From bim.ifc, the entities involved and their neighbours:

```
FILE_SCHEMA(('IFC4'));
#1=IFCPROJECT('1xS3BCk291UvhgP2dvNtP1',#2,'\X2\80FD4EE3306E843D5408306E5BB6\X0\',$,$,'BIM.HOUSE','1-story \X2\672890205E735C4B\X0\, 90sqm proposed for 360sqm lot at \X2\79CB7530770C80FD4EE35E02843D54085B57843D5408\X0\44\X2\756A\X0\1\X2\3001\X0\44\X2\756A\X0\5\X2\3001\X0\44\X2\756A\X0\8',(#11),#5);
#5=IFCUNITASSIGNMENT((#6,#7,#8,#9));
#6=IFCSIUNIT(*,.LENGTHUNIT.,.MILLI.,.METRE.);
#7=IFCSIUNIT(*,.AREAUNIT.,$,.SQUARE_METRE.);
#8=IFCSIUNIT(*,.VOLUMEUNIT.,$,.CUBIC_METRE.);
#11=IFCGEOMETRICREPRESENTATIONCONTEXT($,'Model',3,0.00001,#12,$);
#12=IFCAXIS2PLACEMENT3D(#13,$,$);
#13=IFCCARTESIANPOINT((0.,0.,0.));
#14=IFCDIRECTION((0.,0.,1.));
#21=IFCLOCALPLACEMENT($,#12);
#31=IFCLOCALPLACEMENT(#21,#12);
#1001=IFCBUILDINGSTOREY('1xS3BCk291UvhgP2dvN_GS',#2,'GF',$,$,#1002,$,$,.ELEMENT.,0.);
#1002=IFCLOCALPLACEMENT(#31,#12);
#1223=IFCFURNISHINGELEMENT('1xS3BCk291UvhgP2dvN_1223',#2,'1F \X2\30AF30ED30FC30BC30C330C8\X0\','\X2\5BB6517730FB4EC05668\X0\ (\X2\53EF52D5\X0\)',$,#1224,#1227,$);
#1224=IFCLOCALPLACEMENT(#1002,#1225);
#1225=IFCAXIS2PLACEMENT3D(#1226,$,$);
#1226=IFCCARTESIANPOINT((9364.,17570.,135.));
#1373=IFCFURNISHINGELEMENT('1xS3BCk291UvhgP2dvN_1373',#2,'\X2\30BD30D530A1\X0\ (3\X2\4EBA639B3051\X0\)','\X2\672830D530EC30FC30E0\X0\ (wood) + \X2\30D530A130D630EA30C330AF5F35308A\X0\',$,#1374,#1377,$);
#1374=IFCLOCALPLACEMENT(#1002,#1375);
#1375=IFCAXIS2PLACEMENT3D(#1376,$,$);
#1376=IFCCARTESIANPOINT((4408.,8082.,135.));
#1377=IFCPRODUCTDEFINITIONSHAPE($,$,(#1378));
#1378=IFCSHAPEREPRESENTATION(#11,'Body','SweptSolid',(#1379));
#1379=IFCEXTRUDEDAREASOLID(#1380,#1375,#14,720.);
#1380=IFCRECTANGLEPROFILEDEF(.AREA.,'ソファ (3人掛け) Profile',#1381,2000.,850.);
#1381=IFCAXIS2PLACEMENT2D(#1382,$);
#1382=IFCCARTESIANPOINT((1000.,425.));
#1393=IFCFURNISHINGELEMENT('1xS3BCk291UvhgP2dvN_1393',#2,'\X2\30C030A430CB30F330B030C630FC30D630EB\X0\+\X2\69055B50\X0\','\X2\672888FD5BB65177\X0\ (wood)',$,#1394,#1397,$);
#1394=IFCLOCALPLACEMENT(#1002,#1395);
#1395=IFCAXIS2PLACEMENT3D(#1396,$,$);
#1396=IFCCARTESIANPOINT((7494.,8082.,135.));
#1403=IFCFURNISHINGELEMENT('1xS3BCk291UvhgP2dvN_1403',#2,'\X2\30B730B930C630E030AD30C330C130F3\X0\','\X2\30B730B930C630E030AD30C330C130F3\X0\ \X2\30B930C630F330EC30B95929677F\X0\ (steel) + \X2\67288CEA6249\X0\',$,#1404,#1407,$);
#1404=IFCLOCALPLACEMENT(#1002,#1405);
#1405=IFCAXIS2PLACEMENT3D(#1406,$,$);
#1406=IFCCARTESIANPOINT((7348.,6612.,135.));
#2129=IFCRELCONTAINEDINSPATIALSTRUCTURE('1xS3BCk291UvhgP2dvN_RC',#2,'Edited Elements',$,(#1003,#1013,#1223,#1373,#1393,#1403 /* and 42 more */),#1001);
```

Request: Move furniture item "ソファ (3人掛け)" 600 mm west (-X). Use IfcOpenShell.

```python
import ifcopenshell
import ifcopenshell.api.geometry
import ifcopenshell.util.placement

model = ifcopenshell.open("bim.ifc")

item = model.by_guid("1xS3BCk291UvhgP2dvN_1373")
matrix = ifcopenshell.util.placement.get_local_placement(item.ObjectPlacement)
matrix[0, 3] -= 600.0
ifcopenshell.api.geometry.edit_object_placement(model, product=item, matrix=matrix, is_si=False)

print(ifcopenshell.util.placement.get_local_placement(item.ObjectPlacement).round(3) + 0.0)

model.write("bim_updated.ifc")
```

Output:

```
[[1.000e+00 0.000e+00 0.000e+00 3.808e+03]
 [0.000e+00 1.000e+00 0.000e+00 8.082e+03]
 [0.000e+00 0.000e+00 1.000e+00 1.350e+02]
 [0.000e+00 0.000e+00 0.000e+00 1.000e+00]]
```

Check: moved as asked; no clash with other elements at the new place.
